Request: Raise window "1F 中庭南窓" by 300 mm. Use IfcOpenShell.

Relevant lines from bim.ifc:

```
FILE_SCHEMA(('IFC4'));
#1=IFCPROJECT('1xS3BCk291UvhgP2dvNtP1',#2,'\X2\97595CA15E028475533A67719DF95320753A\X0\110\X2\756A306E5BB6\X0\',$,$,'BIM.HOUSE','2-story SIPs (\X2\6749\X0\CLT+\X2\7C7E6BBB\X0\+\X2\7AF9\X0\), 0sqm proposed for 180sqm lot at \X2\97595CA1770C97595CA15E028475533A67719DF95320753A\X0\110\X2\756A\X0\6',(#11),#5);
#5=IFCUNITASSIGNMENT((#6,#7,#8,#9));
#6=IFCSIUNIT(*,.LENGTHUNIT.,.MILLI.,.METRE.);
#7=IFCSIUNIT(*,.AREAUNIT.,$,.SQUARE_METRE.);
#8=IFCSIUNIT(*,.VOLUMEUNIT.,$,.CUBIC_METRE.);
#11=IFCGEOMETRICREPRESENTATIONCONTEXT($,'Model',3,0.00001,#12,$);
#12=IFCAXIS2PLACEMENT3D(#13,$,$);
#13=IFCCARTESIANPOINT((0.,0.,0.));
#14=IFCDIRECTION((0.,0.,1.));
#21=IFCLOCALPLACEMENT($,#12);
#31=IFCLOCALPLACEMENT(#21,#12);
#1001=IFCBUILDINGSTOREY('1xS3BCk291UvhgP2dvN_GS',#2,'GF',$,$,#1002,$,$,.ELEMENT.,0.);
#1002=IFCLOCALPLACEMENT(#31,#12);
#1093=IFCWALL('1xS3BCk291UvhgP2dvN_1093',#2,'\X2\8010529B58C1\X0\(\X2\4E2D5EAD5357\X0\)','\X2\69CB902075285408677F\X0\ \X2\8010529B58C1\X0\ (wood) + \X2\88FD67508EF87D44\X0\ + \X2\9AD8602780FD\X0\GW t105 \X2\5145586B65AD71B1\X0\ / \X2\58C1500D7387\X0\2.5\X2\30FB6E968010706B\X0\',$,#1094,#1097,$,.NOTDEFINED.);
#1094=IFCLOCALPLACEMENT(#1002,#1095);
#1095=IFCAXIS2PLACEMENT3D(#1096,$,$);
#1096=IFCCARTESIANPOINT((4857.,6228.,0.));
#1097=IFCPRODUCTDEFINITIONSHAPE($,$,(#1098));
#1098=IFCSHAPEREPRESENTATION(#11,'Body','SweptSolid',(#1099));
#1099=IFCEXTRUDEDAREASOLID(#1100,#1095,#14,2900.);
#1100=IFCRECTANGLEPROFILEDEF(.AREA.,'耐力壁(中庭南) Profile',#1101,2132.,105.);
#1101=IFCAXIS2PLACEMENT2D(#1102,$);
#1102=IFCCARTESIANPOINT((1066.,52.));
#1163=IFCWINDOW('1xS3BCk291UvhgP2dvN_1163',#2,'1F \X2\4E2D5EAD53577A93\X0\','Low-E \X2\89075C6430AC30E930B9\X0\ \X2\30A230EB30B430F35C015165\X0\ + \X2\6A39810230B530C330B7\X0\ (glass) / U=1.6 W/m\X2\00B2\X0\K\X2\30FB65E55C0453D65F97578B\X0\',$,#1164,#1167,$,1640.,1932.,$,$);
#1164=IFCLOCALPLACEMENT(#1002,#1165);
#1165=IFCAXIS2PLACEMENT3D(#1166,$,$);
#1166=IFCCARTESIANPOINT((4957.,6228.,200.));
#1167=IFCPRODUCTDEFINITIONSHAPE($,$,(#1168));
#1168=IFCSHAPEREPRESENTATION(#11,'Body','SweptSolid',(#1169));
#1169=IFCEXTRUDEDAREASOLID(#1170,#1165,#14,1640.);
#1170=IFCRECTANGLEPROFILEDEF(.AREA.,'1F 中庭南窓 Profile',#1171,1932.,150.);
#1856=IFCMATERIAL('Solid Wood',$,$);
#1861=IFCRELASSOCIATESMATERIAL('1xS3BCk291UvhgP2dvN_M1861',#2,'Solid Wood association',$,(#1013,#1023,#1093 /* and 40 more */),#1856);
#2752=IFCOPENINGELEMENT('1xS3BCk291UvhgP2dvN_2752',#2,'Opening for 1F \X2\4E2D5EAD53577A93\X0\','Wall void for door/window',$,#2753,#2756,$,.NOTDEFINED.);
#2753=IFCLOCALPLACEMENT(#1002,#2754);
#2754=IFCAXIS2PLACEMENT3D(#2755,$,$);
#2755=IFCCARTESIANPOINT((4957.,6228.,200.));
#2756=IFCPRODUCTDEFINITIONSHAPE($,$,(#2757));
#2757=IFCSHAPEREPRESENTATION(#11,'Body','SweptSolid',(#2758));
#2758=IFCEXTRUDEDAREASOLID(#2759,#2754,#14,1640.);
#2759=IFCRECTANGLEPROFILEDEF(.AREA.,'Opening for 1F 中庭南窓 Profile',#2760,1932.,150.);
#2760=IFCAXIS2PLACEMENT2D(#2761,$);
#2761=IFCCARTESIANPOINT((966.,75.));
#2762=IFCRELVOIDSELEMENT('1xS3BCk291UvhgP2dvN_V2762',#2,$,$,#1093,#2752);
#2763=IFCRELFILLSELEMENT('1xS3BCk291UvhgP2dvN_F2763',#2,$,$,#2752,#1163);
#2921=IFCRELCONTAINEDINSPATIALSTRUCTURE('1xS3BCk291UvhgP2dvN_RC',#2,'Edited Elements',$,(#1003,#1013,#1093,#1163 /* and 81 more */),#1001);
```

```python
import numpy as np
import ifcopenshell
import ifcopenshell.api.geometry
import ifcopenshell.util.placement
import ifcopenshell.util.unit

model = ifcopenshell.open("bim.ifc")
unit_scale = ifcopenshell.util.unit.calculate_unit_scale(model)

window = model.by_guid("1xS3BCk291UvhgP2dvN_1163")
opening = window.FillsVoids[0].RelatingOpeningElement
dz = 0.3 / unit_scale

shift = np.array([0.0, 0.0, dz])
# The window is not placed relative to its opening, so move both.
for product in (opening, window):
    matrix = ifcopenshell.util.placement.get_local_placement(product.ObjectPlacement)
    matrix[:3, 3] += shift
    ifcopenshell.api.geometry.edit_object_placement(model, product=product, matrix=matrix, is_si=False)

print(f"moved by {dz * unit_scale:+.3f} m")

model.write("bim_rev.ifc")
```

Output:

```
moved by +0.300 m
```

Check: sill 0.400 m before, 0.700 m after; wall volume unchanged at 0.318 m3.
